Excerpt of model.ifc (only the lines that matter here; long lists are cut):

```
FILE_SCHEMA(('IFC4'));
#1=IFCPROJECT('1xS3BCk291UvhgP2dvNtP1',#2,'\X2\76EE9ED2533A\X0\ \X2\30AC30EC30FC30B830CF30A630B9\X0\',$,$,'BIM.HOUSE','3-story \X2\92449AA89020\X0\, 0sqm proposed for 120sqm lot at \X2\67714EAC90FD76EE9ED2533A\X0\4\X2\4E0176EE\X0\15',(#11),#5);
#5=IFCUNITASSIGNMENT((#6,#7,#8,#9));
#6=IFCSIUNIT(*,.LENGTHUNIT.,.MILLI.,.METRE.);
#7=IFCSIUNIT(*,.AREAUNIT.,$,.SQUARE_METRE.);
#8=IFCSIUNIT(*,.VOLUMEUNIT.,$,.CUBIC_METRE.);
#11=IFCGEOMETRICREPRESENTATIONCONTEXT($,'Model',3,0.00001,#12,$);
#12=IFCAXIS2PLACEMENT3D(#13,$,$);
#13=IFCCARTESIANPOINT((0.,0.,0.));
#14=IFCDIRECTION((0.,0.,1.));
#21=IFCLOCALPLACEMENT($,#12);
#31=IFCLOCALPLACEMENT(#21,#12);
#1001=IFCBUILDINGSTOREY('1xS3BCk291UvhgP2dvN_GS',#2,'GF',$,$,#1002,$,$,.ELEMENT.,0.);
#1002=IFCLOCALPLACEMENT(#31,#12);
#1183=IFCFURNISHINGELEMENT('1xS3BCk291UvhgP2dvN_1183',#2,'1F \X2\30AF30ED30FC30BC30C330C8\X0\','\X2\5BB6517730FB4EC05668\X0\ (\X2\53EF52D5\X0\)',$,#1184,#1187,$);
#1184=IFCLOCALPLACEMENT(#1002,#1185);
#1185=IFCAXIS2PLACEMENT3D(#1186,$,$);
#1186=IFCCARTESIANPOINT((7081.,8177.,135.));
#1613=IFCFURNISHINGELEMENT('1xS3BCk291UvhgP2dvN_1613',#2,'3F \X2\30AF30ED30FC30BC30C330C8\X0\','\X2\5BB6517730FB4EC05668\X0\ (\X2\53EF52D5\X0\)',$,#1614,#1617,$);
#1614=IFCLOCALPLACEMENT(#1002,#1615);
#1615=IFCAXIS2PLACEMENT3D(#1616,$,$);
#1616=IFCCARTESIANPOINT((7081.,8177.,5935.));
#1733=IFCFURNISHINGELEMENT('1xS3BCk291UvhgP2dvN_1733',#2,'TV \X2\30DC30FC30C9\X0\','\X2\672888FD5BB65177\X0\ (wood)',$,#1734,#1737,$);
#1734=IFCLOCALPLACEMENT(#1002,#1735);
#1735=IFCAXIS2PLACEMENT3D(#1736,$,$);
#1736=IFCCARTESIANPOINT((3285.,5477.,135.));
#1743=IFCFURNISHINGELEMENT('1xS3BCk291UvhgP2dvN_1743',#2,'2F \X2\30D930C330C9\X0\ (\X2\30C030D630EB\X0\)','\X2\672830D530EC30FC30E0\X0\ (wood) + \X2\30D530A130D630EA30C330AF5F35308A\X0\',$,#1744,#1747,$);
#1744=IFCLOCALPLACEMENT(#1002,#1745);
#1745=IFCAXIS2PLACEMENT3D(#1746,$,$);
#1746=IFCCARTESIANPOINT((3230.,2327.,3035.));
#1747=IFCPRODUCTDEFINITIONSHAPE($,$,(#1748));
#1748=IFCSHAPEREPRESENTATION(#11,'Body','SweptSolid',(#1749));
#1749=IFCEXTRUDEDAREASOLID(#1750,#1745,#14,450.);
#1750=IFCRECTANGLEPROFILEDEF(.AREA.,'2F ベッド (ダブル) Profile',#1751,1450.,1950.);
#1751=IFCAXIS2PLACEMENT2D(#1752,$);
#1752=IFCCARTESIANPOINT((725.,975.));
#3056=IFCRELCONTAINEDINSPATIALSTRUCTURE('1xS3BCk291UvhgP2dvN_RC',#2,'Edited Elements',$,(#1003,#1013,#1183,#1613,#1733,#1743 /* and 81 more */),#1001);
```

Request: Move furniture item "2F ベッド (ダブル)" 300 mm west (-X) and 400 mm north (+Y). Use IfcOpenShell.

```python
import ifcopenshell
import ifcopenshell.api.geometry
import ifcopenshell.util.placement

model = ifcopenshell.open("model.ifc")

item = model.by_id(1743)
matrix = ifcopenshell.util.placement.get_local_placement(item.ObjectPlacement)
matrix[0, 3] -= 300.0
matrix[1, 3] += 400.0
ifcopenshell.api.geometry.edit_object_placement(model, product=item, matrix=matrix, is_si=False)

print(ifcopenshell.util.placement.get_local_placement(item.ObjectPlacement).round(3) + 0.0)

model.write("model_v2.ifc")
```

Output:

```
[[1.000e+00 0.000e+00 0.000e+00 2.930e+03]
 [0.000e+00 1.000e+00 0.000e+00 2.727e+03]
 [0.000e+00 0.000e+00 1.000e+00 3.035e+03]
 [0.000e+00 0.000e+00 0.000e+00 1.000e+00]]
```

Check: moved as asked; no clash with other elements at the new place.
